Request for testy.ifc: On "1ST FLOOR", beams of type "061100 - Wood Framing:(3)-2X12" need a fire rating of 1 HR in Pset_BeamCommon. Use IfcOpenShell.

First a look at what the model holds.

```python
import ifcopenshell
import ifcopenshell.util.element

model = ifcopenshell.open("testy.ifc")
print(model.schema)
storey = next(s for s in model.by_type("IfcBuildingStorey") if s.Name == "1ST FLOOR")
beams = [e for e in ifcopenshell.util.element.get_decomposition(storey) if e.is_a("IfcBeam")]
seen = {}
for e in beams:
    element_type = ifcopenshell.util.element.get_type(e)
    key = (element_type.Name if element_type != e and element_type else None, ifcopenshell.util.element.get_pset(e, "Pset_BeamCommon", "FireRating"))
    seen[key] = seen.get(key, 0) + 1
for (name, value), count in sorted(seen.items(), key=str):
    print(count, "x", name, "|", value)
```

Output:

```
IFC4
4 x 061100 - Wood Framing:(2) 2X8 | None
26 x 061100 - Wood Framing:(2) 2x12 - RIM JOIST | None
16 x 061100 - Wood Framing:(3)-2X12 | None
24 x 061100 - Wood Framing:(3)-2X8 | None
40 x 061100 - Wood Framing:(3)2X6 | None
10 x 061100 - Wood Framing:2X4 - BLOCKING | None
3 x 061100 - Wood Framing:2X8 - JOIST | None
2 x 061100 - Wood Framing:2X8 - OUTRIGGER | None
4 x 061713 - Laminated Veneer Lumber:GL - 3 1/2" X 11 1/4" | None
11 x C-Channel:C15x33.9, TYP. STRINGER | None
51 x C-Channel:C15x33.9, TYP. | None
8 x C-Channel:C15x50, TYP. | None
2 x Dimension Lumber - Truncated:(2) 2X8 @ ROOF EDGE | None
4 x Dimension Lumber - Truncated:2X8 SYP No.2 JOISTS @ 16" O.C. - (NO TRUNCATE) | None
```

```python
import ifcopenshell
import ifcopenshell.api.pset
import ifcopenshell.util.element

model = ifcopenshell.open("testy.ifc")

storey = next(s for s in model.by_type("IfcBuildingStorey") if s.Name == "1ST FLOOR")
beams = [e for e in ifcopenshell.util.element.get_decomposition(storey) if e.is_a("IfcBeam")]

count = 0
for e in beams:
    element_type = ifcopenshell.util.element.get_type(e)
    if element_type in (None, e) or element_type.Name != "061100 - Wood Framing:(3)-2X12":
        continue
    # add_pset returns the element's existing set when there is one.
    pset = ifcopenshell.api.pset.add_pset(model, product=e, name="Pset_BeamCommon")
    ifcopenshell.api.pset.edit_pset(model, pset=pset, properties={"FireRating": "1 HR"})
    count += 1

print(count, "beams updated")

model.write("testy_updated.ifc")
```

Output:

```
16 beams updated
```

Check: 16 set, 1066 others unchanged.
